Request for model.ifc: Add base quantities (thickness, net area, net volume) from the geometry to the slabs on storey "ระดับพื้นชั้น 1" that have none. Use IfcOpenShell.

First a look at what the model holds.

```python
import ifcopenshell
import ifcopenshell.util.element
import ifcopenshell.util.unit

model = ifcopenshell.open("model.ifc")
print(model.schema)
for unit_type in ("LENGTHUNIT", "AREAUNIT", "VOLUMEUNIT"):
    print(unit_type, ifcopenshell.util.unit.calculate_unit_scale(model, unit_type))
storey = next(s for s in model.by_type("IfcBuildingStorey") if s.Name == "ระดับพื้นชั้น 1")
slabs = [e for e in ifcopenshell.util.element.get_decomposition(storey) if e.is_a("IfcSlab")]
for e in sorted(slabs, key=lambda e: e.id()):
    print(e.id(), e.is_a(), e.Name, list(ifcopenshell.util.element.get_psets(e, qtos_only=True)), sep=" | ")
```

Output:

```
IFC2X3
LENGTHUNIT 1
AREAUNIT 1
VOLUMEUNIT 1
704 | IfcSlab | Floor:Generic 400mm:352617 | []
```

```python
import ifcopenshell
import ifcopenshell.api.pset
import ifcopenshell.geom
import ifcopenshell.util.element
import ifcopenshell.util.shape
import ifcopenshell.util.unit

model = ifcopenshell.open("model.ifc")
unit_scale = ifcopenshell.util.unit.calculate_unit_scale(model)
area_scale = ifcopenshell.util.unit.calculate_unit_scale(model, "AREAUNIT")
volume_scale = ifcopenshell.util.unit.calculate_unit_scale(model, "VOLUMEUNIT")
settings = ifcopenshell.geom.settings()

storey = next(s for s in model.by_type("IfcBuildingStorey") if s.Name == "ระดับพื้นชั้น 1")
slabs = [e for e in ifcopenshell.util.element.get_decomposition(storey) if e.is_a("IfcSlab")]

for e in sorted(slabs, key=lambda e: e.id()):
    if ifcopenshell.util.element.get_psets(e, qtos_only=True, should_inherit=False):
        continue
    # Geometry comes back in metres, in the element's own axes.
    shape = ifcopenshell.geom.create_shape(settings, e)
    values = {
        "Width": ifcopenshell.util.shape.get_z(shape.geometry) / unit_scale,
        "NetArea": ifcopenshell.util.shape.get_footprint_area(shape.geometry) / area_scale,
        "NetVolume": ifcopenshell.util.shape.get_volume(shape.geometry) / volume_scale,
    }
    qto = ifcopenshell.api.pset.add_qto(model, product=e, name="BaseQuantities")
    ifcopenshell.api.pset.edit_qto(model, qto=qto, properties=values)
    print(e.id(), {k: round(v, 3) for k, v in values.items()})

model.write("model_edited.ifc")
```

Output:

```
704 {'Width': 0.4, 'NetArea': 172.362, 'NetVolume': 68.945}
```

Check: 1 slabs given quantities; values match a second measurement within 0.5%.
